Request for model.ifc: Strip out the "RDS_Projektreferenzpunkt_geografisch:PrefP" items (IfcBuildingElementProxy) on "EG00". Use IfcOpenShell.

First a look at what the model holds.

```python
import ifcopenshell
import ifcopenshell.util.element

model = ifcopenshell.open("model.ifc")
print(model.schema)
storey = next(s for s in model.by_type("IfcBuildingStorey") if s.Name == "EG00")
proxies = [e for e in ifcopenshell.util.element.get_decomposition(storey) if e.is_a("IfcBuildingElementProxy")]
seen = {}
for e in proxies:
    element_type = ifcopenshell.util.element.get_type(e)
    name = element_type.Name if element_type not in (None, e) else None
    seen[name] = seen.get(name, 0) + 1
for name, count in sorted(seen.items(), key=str):
    print(count, "x", name)
```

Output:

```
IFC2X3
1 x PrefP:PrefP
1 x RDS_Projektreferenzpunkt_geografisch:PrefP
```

```python
import ifcopenshell
import ifcopenshell.api.root
import ifcopenshell.util.element

model = ifcopenshell.open("model.ifc")

storey = next(s for s in model.by_type("IfcBuildingStorey") if s.Name == "EG00")
proxies = [e for e in ifcopenshell.util.element.get_decomposition(storey) if e.is_a("IfcBuildingElementProxy")]
targets = [e for e in proxies if (t := ifcopenshell.util.element.get_type(e)) not in (None, e) and t.Name == "RDS_Projektreferenzpunkt_geografisch:PrefP"]

for e in targets:
    ifcopenshell.api.root.remove_product(model, product=e)
print(len(targets), "removed")

model.write("model_v2.ifc")
```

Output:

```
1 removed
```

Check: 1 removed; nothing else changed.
